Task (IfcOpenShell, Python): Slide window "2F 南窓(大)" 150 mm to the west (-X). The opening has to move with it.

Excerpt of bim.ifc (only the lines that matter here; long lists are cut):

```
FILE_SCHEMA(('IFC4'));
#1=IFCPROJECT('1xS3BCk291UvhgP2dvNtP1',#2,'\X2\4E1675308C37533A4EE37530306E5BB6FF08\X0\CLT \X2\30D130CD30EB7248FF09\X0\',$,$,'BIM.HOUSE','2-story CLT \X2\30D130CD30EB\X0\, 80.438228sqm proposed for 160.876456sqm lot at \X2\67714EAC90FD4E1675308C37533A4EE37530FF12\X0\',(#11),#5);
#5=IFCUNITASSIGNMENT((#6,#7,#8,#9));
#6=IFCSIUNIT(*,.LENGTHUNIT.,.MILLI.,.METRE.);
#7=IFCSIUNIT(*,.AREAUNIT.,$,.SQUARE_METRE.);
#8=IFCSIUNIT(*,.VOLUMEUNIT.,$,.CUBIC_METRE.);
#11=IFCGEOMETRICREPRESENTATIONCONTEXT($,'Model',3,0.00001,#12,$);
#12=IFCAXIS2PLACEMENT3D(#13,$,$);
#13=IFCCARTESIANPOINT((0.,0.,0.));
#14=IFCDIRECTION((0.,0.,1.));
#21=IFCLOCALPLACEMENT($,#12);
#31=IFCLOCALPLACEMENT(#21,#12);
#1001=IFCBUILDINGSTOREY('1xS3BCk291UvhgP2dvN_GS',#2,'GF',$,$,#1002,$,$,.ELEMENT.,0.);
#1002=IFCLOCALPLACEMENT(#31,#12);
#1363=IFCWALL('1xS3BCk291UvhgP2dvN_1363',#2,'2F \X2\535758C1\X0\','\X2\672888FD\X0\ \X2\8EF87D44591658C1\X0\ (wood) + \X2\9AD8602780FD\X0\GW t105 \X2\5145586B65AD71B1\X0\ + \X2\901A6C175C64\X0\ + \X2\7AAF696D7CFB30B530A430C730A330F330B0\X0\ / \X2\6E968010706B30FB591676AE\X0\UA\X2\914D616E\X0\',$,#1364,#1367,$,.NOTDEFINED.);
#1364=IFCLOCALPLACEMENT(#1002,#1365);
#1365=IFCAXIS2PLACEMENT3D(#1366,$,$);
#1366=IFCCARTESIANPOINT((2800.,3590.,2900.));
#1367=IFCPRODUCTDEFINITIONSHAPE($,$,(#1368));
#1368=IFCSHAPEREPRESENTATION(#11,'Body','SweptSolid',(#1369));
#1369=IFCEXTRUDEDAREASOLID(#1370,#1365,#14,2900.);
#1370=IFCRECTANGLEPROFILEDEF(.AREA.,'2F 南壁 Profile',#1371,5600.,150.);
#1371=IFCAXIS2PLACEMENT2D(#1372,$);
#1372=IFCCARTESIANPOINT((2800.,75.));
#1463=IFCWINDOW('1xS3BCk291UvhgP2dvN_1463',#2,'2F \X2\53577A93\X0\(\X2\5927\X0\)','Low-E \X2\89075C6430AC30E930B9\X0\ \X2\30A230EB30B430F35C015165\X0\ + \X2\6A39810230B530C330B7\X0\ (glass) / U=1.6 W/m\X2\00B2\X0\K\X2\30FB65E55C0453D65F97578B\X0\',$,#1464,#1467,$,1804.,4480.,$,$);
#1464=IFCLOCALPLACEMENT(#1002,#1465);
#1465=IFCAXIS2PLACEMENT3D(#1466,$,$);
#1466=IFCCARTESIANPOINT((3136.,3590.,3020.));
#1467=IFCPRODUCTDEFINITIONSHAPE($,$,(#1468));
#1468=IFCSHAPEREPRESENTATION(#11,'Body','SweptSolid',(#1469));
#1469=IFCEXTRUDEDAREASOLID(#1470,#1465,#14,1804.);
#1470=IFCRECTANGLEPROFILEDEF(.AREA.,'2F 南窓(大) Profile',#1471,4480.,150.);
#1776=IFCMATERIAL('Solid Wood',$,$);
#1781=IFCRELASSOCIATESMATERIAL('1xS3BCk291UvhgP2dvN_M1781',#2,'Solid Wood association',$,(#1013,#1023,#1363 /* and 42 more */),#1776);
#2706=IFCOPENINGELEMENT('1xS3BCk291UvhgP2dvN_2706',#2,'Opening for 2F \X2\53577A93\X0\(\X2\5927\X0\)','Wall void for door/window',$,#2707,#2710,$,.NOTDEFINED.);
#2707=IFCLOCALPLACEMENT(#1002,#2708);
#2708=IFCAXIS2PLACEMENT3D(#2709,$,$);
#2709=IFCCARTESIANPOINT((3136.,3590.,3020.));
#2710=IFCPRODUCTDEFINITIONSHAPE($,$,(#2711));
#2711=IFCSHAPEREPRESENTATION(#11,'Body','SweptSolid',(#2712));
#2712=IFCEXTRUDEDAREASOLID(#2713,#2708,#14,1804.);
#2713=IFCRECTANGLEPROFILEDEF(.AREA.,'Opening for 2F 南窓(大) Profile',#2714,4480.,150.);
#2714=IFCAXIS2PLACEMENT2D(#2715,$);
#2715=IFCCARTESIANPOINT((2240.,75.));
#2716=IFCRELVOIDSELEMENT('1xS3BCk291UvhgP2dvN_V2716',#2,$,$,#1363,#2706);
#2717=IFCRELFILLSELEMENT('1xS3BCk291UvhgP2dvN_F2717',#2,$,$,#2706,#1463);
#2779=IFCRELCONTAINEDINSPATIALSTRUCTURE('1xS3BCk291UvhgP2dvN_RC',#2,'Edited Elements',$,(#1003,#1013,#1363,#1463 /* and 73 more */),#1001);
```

```python
import ifcopenshell
import ifcopenshell.api.geometry
import ifcopenshell.util.placement
import ifcopenshell.util.unit

model = ifcopenshell.open("bim.ifc")
unit_scale = ifcopenshell.util.unit.calculate_unit_scale(model)

window = model.by_guid("1xS3BCk291UvhgP2dvN_1463")
opening = window.FillsVoids[0].RelatingOpeningElement
wall = opening.VoidsElements[0].RelatingBuildingElement

wall_matrix = ifcopenshell.util.placement.get_local_placement(wall.ObjectPlacement)
shift = wall_matrix[:3, 0] * -0.15 / unit_scale
before = ifcopenshell.util.placement.get_local_placement(window.ObjectPlacement)[:3, 3].copy()

# The window is not placed relative to its opening, so move both.
for product in (opening, window):
    matrix = ifcopenshell.util.placement.get_local_placement(product.ObjectPlacement)
    matrix[:3, 3] += shift
    ifcopenshell.api.geometry.edit_object_placement(model, product=product, matrix=matrix, is_si=False)

after = ifcopenshell.util.placement.get_local_placement(window.ObjectPlacement)[:3, 3]
print("window moved by", (after - before).round(3) + 0.0)

model.write("bim_edited.ifc")
```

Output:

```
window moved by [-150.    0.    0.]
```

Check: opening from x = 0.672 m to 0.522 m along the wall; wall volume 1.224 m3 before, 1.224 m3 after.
